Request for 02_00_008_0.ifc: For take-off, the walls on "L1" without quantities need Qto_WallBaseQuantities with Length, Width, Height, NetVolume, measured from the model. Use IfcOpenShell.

First a look at what the model holds.

```python
import ifcopenshell
import ifcopenshell.util.element
import ifcopenshell.util.unit

model = ifcopenshell.open("02_00_008_0.ifc")
print(model.schema)
for unit_type in ("LENGTHUNIT", "AREAUNIT", "VOLUMEUNIT"):
    print(unit_type, ifcopenshell.util.unit.calculate_unit_scale(model, unit_type))
storey = next(s for s in model.by_type("IfcBuildingStorey") if s.Name == "L1")
walls = [e for e in ifcopenshell.util.element.get_decomposition(storey) if e.is_a("IfcWall")]
for e in sorted(walls, key=lambda e: e.id()):
    print(e.id(), e.is_a(), e.Name, list(ifcopenshell.util.element.get_psets(e, qtos_only=True)), sep=" | ")
```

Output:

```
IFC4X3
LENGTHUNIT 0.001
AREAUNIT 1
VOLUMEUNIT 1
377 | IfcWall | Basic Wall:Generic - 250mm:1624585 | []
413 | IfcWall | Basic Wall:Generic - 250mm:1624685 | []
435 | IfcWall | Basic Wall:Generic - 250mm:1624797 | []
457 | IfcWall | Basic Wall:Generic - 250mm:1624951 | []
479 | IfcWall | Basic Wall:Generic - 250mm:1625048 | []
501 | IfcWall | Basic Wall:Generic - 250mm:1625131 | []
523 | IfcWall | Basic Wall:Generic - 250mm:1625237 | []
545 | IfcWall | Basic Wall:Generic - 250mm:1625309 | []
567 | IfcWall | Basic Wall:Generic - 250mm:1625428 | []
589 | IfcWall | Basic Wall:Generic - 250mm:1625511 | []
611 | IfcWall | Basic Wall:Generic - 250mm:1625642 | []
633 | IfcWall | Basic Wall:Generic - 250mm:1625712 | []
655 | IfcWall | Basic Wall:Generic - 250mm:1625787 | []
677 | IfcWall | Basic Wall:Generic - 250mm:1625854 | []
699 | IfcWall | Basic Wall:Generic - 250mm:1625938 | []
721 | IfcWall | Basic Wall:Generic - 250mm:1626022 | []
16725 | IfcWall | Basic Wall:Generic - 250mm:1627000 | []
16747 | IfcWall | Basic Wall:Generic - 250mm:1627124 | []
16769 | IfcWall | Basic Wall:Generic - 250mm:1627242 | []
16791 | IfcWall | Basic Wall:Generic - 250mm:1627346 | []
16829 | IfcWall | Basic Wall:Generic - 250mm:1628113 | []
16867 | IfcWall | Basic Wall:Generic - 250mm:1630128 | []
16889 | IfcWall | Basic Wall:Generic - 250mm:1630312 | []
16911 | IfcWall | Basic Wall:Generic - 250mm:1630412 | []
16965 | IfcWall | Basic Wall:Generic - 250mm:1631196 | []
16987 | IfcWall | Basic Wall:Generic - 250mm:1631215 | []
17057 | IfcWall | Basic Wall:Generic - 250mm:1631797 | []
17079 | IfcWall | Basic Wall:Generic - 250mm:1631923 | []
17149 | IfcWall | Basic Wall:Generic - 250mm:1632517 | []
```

```python
import ifcopenshell
import ifcopenshell.api.pset
import ifcopenshell.geom
import ifcopenshell.util.element
import ifcopenshell.util.shape
import ifcopenshell.util.unit

model = ifcopenshell.open("02_00_008_0.ifc")
unit_scale = ifcopenshell.util.unit.calculate_unit_scale(model)
volume_scale = ifcopenshell.util.unit.calculate_unit_scale(model, "VOLUMEUNIT")
settings = ifcopenshell.geom.settings()

storey = next(s for s in model.by_type("IfcBuildingStorey") if s.Name == "L1")
walls = [e for e in ifcopenshell.util.element.get_decomposition(storey) if e.is_a("IfcWall")]

for e in sorted(walls, key=lambda e: e.id()):
    if ifcopenshell.util.element.get_psets(e, qtos_only=True, should_inherit=False):
        continue
    # Geometry comes back in metres, in the element's own axes.
    shape = ifcopenshell.geom.create_shape(settings, e)
    values = {
        "Length": ifcopenshell.util.shape.get_x(shape.geometry) / unit_scale,
        "Width": ifcopenshell.util.shape.get_y(shape.geometry) / unit_scale,
        "Height": ifcopenshell.util.shape.get_z(shape.geometry) / unit_scale,
        "NetVolume": ifcopenshell.util.shape.get_volume(shape.geometry) / volume_scale,
    }
    qto = ifcopenshell.api.pset.add_qto(model, product=e, name="Qto_WallBaseQuantities")
    ifcopenshell.api.pset.edit_qto(model, qto=qto, properties=values)
    print(e.id(), {k: round(v, 3) for k, v in values.items()})

model.write("02_00_008_0-out.ifc")
```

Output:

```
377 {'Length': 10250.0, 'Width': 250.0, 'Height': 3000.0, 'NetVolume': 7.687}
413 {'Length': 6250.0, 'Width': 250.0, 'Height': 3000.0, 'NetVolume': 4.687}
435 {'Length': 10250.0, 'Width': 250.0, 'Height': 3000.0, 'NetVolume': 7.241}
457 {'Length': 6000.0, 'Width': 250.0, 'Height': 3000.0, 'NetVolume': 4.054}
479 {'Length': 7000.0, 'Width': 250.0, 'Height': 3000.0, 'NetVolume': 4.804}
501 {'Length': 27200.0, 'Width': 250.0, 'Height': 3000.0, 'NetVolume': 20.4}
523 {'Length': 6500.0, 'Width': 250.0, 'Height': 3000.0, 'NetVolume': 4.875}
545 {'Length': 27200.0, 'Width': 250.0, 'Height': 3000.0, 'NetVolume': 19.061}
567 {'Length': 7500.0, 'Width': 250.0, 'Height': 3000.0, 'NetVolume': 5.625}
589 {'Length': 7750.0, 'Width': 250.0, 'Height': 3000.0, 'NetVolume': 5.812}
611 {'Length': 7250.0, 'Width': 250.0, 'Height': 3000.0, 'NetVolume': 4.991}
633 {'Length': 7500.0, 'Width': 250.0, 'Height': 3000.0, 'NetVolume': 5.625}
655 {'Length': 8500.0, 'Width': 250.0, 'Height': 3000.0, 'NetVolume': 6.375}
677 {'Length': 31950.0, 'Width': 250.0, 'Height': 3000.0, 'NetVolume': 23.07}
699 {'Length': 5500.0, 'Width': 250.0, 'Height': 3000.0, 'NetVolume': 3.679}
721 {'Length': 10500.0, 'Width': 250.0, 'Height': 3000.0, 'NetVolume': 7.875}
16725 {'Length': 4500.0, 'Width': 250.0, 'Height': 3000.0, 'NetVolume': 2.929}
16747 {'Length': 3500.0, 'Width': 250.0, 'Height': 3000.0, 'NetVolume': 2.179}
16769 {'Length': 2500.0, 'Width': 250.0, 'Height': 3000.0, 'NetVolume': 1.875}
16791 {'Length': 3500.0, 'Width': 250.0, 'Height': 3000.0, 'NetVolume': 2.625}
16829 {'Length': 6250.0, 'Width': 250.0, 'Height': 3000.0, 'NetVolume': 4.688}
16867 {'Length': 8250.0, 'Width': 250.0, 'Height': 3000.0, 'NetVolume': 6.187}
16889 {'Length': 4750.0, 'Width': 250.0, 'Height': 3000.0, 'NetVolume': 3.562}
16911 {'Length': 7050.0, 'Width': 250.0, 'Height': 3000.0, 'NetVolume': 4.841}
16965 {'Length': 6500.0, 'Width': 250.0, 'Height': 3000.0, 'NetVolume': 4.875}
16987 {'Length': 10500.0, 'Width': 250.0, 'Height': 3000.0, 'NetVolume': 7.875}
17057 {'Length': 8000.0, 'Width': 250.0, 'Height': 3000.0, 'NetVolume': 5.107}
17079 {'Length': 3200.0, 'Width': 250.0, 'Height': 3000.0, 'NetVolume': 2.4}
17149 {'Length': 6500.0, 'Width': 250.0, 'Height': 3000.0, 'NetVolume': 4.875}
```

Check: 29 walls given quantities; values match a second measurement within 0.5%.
